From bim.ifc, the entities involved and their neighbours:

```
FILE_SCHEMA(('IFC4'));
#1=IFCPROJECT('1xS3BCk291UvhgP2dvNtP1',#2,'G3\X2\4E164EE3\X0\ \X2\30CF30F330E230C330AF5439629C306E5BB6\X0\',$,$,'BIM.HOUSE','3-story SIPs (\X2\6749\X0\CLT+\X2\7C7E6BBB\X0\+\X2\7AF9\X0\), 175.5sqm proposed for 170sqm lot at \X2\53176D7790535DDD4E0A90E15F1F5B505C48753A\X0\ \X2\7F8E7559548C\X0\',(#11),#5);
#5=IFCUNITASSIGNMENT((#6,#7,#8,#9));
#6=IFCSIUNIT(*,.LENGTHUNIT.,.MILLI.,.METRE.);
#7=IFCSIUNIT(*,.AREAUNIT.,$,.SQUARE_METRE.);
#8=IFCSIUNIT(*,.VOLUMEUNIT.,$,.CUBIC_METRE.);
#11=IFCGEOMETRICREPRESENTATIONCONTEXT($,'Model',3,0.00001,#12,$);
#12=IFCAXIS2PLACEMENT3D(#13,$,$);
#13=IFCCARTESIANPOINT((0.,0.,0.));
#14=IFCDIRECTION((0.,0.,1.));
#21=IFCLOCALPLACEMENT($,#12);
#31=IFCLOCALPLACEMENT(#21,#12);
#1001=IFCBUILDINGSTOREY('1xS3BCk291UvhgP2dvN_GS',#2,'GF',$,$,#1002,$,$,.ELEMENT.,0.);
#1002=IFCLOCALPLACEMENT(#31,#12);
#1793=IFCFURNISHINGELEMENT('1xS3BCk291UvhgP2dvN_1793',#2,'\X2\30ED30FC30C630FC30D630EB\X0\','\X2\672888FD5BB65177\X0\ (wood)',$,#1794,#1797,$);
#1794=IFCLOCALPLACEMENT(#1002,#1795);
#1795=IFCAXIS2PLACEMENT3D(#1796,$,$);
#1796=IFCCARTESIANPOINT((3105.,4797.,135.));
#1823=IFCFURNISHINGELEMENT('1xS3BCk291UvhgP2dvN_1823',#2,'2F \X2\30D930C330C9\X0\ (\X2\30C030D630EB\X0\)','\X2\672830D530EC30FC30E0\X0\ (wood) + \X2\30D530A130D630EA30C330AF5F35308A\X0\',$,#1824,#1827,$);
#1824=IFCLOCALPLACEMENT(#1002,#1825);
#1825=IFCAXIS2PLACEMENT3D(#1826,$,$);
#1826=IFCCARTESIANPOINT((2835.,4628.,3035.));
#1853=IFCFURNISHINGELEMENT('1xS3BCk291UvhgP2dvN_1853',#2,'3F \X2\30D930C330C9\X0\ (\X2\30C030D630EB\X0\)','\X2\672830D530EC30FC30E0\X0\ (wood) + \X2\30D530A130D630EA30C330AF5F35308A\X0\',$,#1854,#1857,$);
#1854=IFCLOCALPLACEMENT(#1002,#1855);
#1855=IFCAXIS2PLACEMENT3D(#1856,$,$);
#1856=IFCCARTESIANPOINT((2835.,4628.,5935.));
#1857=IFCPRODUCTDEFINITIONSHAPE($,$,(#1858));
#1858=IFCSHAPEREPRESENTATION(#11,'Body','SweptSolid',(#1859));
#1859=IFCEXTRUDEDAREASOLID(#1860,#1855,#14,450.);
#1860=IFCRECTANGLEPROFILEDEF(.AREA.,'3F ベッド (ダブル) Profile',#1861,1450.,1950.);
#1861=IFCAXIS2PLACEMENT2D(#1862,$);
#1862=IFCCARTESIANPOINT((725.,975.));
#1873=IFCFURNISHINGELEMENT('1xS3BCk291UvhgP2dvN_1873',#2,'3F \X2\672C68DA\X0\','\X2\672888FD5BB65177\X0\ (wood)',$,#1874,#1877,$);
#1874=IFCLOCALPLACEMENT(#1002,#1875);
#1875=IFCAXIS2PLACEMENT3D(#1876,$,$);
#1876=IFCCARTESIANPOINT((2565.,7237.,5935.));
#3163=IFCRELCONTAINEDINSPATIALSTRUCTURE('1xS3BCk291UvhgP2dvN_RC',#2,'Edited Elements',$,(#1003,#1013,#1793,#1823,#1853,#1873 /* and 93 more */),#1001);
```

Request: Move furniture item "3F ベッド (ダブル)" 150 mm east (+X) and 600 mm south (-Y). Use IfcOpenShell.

```python
import ifcopenshell
import ifcopenshell.api.geometry
import ifcopenshell.util.placement
import ifcopenshell.util.unit

model = ifcopenshell.open("bim.ifc")
unit_scale = ifcopenshell.util.unit.calculate_unit_scale(model)

item = model.by_guid("1xS3BCk291UvhgP2dvN_1853")
matrix = ifcopenshell.util.placement.get_local_placement(item.ObjectPlacement)
matrix[0, 3] += 0.15 / unit_scale
matrix[1, 3] -= 0.6 / unit_scale
ifcopenshell.api.geometry.edit_object_placement(model, product=item, matrix=matrix, is_si=False)

print(ifcopenshell.util.placement.get_local_placement(item.ObjectPlacement).round(3) + 0.0)

model.write("bim_v2.ifc")
```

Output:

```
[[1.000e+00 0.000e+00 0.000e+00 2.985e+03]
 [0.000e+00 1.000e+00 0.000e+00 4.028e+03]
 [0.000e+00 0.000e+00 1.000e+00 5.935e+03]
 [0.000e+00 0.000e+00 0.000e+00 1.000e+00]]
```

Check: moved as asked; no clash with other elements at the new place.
